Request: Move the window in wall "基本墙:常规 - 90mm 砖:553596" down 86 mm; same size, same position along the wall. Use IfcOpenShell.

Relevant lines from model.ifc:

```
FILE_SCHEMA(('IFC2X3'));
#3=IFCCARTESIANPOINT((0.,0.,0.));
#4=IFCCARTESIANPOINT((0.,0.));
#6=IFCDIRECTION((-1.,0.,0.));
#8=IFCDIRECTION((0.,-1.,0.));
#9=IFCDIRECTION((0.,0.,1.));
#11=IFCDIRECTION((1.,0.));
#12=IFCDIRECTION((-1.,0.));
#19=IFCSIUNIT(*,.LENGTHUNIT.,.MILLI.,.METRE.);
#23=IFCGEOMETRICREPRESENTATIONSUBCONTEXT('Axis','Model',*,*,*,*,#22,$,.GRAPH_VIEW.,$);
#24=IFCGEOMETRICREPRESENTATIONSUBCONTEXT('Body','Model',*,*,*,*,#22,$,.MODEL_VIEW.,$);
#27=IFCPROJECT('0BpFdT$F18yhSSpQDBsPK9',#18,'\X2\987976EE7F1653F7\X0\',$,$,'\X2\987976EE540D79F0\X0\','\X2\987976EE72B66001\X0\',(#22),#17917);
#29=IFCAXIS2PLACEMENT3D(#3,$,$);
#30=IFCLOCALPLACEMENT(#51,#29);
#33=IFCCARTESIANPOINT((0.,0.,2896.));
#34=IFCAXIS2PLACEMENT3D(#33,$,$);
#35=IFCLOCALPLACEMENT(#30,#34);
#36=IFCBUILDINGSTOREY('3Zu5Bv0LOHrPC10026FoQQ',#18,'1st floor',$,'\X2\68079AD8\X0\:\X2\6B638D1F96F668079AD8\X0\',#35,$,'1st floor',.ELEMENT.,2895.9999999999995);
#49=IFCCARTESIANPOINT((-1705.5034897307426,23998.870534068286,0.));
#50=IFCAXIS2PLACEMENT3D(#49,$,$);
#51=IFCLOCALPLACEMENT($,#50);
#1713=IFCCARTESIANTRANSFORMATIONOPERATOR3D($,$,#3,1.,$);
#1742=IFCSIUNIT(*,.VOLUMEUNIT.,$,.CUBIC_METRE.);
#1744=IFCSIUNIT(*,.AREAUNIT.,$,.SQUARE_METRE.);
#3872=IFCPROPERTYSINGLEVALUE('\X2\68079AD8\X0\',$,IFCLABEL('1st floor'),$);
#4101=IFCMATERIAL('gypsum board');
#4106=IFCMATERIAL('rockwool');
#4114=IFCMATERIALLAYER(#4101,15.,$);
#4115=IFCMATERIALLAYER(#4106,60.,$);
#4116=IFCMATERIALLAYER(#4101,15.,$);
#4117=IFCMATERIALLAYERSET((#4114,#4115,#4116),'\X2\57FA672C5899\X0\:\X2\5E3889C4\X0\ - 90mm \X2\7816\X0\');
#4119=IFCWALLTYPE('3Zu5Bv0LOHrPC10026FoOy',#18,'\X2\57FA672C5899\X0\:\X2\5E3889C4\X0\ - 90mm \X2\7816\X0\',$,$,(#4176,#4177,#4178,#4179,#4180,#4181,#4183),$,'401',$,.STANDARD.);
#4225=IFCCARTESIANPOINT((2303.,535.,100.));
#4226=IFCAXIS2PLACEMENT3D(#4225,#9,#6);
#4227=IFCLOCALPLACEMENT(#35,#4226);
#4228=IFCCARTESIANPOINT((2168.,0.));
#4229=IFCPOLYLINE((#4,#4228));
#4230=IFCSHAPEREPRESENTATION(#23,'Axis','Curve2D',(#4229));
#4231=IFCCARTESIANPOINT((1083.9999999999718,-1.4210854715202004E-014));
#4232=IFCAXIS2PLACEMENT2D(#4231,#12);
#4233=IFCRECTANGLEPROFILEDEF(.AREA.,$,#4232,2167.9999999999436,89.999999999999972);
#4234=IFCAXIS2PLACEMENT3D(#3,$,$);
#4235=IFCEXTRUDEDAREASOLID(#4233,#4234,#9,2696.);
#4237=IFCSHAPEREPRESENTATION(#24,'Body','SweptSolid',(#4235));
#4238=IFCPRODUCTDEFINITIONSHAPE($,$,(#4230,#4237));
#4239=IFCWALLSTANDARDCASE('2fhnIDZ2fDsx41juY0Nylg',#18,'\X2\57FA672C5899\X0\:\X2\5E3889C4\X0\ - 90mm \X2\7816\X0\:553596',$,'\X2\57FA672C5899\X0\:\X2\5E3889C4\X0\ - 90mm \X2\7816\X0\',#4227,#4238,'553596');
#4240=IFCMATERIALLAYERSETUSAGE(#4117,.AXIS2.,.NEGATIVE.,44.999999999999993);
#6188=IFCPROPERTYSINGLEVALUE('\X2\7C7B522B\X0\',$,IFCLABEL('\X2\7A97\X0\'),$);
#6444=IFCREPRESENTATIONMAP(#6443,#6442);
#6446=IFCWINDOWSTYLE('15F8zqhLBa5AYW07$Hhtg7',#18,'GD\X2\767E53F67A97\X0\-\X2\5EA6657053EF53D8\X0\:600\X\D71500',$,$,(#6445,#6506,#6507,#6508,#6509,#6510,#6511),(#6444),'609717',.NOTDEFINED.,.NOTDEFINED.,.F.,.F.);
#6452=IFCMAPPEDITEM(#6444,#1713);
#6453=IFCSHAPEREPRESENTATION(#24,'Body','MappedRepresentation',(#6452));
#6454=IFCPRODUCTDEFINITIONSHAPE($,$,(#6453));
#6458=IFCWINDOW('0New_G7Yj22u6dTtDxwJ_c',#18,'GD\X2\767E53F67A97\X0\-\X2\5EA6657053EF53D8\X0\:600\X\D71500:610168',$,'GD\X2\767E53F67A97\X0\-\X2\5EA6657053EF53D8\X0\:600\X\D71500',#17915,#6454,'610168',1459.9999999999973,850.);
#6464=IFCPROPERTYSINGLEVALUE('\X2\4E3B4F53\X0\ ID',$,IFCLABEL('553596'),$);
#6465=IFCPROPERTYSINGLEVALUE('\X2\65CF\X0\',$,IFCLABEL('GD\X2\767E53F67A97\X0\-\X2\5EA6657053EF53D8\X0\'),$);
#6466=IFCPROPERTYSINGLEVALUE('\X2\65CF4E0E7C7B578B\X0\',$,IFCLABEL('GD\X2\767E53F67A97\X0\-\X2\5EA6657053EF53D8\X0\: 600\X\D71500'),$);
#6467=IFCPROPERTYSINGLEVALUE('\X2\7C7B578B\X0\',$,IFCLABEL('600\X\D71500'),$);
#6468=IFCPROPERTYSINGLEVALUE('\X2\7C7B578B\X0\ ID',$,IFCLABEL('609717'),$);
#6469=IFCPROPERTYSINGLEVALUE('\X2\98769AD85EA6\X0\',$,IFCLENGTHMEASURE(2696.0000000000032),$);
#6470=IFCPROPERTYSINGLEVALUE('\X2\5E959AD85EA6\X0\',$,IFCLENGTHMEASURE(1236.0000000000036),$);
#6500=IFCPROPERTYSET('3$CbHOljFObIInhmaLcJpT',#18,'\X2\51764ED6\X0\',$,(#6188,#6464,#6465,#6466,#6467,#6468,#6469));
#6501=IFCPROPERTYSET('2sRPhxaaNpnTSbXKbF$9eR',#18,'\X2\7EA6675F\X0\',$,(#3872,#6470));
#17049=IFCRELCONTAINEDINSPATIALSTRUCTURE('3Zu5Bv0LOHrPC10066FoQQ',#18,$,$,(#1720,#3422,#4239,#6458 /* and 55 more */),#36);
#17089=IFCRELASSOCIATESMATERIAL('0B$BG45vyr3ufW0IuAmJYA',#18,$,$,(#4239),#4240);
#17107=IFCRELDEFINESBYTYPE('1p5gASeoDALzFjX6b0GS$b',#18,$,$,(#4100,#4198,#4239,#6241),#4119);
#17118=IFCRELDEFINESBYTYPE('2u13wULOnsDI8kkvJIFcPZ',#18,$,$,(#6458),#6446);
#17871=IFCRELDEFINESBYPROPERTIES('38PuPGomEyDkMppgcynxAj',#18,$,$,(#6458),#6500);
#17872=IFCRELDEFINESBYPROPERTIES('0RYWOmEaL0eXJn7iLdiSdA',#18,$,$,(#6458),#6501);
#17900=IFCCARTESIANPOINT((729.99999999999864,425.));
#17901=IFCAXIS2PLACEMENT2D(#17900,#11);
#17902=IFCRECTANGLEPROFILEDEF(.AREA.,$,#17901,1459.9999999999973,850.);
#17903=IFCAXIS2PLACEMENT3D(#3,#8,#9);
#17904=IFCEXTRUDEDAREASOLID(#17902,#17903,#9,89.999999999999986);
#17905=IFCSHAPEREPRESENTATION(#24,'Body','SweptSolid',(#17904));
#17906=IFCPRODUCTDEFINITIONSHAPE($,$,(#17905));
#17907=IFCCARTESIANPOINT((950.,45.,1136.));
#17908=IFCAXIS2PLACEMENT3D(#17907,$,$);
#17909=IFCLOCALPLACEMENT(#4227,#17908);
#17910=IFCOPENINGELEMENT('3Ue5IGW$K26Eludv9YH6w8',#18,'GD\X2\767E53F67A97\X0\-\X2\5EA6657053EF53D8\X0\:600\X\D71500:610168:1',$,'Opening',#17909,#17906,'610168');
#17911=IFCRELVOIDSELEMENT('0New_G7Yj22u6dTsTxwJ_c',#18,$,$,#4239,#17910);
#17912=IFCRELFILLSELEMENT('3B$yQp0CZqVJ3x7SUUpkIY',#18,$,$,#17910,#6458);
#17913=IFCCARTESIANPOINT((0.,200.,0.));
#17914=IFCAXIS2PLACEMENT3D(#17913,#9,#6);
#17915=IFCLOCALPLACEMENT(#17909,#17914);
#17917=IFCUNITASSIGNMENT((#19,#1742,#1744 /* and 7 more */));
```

```python
import numpy as np
import ifcopenshell
import ifcopenshell.api.geometry
import ifcopenshell.api.pset
import ifcopenshell.util.element
import ifcopenshell.util.placement
import ifcopenshell.util.unit

model = ifcopenshell.open("model.ifc")
unit_scale = ifcopenshell.util.unit.calculate_unit_scale(model)

window = model.by_id(6458)
opening = window.FillsVoids[0].RelatingOpeningElement
dz = -86.0

shift = np.array([0.0, 0.0, dz])
# The window is placed relative to its opening, so it follows when the opening moves.
matrix = ifcopenshell.util.placement.get_local_placement(opening.ObjectPlacement)
matrix[:3, 3] += shift
ifcopenshell.api.geometry.edit_object_placement(
    model, product=opening, matrix=matrix, is_si=False, should_transform_children=True
)

# Keep the stored heights in step.
pset = model.by_id(ifcopenshell.util.element.get_pset(window, "其他", should_inherit=False)["id"])
ifcopenshell.api.pset.edit_pset(model, pset=pset, properties={
    "顶高度": model.create_entity("IfcLengthMeasure", ifcopenshell.util.element.get_pset(window, "其他", "顶高度") + dz),
})
pset = model.by_id(ifcopenshell.util.element.get_pset(window, "约束", should_inherit=False)["id"])
ifcopenshell.api.pset.edit_pset(model, pset=pset, properties={
    "底高度": model.create_entity("IfcLengthMeasure", ifcopenshell.util.element.get_pset(window, "约束", "底高度") + dz),
})

print(f"moved by {dz * unit_scale:+.3f} m")

model.write("model_v2.ifc")
```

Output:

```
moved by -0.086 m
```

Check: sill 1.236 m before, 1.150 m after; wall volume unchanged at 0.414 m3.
